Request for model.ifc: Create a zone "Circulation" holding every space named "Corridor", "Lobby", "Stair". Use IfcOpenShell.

First a look at what the model holds.

```python
import ifcopenshell

model = ifcopenshell.open("model.ifc")
print(model.schema)
seen = {}
for space in model.by_type("IfcSpace"):
    seen[space.LongName] = seen.get(space.LongName, 0) + 1
for name, count in sorted(seen.items(), key=str):
    print(count, "x", name)
print("zones:", [z.Name for z in model.by_type("IfcZone")][:20])
```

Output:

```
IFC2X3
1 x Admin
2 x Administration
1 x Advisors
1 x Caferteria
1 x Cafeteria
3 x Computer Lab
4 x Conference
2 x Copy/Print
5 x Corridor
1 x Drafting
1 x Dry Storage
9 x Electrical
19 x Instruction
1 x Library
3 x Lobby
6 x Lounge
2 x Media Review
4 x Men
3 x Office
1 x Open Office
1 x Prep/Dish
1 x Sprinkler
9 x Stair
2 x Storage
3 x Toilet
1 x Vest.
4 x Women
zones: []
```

```python
import ifcopenshell
import ifcopenshell.api.group
import ifcopenshell.api.root

model = ifcopenshell.open("model.ifc")

names = {"Corridor", "Lobby", "Stair"}
spaces = [s for s in model.by_type("IfcSpace") if s.LongName in names]

zone = ifcopenshell.api.root.create_entity(model, ifc_class="IfcZone", name="Circulation")
ifcopenshell.api.group.assign_group(model, products=spaces, group=zone)
print(len(spaces), "spaces in", zone.Name)

model.write("model_v2.ifc")
```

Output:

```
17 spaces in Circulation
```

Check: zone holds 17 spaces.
